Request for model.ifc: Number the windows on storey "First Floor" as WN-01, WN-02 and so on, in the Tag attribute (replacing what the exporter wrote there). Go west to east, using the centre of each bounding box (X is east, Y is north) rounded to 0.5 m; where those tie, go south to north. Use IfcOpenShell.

First a look at what the model holds.

```python
import ifcopenshell
import ifcopenshell.util.element
import ifcopenshell.util.placement

model = ifcopenshell.open("model.ifc")
print(model.schema)
storey = next(s for s in model.by_type("IfcBuildingStorey") if s.Name == "First Floor")
windows = [e for e in ifcopenshell.util.element.get_decomposition(storey) if e.is_a("IfcWindow")]
for e in sorted(windows, key=lambda e: e.id()):
    origin = ifcopenshell.util.placement.get_local_placement(e.ObjectPlacement)[:3, 3]
    print(e.id(), e.Tag, e.Name, origin.round(2) + 0.0, sep=" | ")
```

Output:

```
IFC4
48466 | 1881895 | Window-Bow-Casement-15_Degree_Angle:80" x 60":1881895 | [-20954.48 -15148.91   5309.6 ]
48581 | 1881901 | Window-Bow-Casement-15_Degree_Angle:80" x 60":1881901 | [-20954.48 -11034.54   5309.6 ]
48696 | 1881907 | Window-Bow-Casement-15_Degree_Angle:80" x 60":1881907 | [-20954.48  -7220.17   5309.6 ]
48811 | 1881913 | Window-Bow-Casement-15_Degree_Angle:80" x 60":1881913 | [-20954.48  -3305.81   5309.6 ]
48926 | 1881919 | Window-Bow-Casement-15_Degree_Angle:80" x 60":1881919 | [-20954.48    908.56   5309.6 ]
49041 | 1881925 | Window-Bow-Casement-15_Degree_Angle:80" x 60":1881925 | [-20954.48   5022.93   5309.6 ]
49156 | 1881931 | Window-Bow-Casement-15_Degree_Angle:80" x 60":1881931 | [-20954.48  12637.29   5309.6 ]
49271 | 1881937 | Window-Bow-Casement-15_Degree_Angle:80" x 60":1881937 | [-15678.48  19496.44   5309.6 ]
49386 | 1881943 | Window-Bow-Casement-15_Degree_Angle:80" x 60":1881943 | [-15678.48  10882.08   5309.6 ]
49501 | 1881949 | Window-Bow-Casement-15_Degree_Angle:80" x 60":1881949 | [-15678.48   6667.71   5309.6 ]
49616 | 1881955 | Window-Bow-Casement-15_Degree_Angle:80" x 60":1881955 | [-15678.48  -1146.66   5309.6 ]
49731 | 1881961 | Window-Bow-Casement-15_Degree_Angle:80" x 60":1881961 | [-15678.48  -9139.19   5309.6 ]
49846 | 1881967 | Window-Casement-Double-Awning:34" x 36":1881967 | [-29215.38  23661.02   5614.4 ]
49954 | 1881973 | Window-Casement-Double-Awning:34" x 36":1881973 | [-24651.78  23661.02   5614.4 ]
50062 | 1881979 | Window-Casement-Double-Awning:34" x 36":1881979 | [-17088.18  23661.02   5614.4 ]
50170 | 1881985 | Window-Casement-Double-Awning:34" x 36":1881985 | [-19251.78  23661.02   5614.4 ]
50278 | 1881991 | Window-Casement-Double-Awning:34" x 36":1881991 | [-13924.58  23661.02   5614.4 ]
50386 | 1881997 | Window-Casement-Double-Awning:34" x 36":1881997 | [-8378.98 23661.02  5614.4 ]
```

```python
import ifcopenshell
import ifcopenshell.geom
import ifcopenshell.util.element
import ifcopenshell.util.shape

model = ifcopenshell.open("model.ifc")
settings = ifcopenshell.geom.settings()
settings.set("use-world-coords", True)


def centre(element):
    shape = ifcopenshell.geom.create_shape(settings, element)
    return ifcopenshell.util.shape.get_bbox_centroid(shape.geometry)


storey = next(s for s in model.by_type("IfcBuildingStorey") if s.Name == "First Floor")
windows = [e for e in ifcopenshell.util.element.get_decomposition(storey) if e.is_a("IfcWindow")]

# Insertion points can sit at a corner or the storey origin, so sort by the geometry (in metres).
centres = {e: centre(e) for e in windows}
windows.sort(key=lambda e: (round(centres[e][0] / 0.5), centres[e][1]))

for i, e in enumerate(windows, start=1):
    number = f"WN-{i:02d}"
    e.Tag = number
    print(e.id(), number)

model.write("model_rev.ifc")
```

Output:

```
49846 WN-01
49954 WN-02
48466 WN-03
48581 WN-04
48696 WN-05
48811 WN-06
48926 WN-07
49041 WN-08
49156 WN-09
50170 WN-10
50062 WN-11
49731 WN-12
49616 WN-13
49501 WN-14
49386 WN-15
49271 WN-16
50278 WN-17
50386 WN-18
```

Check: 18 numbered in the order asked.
